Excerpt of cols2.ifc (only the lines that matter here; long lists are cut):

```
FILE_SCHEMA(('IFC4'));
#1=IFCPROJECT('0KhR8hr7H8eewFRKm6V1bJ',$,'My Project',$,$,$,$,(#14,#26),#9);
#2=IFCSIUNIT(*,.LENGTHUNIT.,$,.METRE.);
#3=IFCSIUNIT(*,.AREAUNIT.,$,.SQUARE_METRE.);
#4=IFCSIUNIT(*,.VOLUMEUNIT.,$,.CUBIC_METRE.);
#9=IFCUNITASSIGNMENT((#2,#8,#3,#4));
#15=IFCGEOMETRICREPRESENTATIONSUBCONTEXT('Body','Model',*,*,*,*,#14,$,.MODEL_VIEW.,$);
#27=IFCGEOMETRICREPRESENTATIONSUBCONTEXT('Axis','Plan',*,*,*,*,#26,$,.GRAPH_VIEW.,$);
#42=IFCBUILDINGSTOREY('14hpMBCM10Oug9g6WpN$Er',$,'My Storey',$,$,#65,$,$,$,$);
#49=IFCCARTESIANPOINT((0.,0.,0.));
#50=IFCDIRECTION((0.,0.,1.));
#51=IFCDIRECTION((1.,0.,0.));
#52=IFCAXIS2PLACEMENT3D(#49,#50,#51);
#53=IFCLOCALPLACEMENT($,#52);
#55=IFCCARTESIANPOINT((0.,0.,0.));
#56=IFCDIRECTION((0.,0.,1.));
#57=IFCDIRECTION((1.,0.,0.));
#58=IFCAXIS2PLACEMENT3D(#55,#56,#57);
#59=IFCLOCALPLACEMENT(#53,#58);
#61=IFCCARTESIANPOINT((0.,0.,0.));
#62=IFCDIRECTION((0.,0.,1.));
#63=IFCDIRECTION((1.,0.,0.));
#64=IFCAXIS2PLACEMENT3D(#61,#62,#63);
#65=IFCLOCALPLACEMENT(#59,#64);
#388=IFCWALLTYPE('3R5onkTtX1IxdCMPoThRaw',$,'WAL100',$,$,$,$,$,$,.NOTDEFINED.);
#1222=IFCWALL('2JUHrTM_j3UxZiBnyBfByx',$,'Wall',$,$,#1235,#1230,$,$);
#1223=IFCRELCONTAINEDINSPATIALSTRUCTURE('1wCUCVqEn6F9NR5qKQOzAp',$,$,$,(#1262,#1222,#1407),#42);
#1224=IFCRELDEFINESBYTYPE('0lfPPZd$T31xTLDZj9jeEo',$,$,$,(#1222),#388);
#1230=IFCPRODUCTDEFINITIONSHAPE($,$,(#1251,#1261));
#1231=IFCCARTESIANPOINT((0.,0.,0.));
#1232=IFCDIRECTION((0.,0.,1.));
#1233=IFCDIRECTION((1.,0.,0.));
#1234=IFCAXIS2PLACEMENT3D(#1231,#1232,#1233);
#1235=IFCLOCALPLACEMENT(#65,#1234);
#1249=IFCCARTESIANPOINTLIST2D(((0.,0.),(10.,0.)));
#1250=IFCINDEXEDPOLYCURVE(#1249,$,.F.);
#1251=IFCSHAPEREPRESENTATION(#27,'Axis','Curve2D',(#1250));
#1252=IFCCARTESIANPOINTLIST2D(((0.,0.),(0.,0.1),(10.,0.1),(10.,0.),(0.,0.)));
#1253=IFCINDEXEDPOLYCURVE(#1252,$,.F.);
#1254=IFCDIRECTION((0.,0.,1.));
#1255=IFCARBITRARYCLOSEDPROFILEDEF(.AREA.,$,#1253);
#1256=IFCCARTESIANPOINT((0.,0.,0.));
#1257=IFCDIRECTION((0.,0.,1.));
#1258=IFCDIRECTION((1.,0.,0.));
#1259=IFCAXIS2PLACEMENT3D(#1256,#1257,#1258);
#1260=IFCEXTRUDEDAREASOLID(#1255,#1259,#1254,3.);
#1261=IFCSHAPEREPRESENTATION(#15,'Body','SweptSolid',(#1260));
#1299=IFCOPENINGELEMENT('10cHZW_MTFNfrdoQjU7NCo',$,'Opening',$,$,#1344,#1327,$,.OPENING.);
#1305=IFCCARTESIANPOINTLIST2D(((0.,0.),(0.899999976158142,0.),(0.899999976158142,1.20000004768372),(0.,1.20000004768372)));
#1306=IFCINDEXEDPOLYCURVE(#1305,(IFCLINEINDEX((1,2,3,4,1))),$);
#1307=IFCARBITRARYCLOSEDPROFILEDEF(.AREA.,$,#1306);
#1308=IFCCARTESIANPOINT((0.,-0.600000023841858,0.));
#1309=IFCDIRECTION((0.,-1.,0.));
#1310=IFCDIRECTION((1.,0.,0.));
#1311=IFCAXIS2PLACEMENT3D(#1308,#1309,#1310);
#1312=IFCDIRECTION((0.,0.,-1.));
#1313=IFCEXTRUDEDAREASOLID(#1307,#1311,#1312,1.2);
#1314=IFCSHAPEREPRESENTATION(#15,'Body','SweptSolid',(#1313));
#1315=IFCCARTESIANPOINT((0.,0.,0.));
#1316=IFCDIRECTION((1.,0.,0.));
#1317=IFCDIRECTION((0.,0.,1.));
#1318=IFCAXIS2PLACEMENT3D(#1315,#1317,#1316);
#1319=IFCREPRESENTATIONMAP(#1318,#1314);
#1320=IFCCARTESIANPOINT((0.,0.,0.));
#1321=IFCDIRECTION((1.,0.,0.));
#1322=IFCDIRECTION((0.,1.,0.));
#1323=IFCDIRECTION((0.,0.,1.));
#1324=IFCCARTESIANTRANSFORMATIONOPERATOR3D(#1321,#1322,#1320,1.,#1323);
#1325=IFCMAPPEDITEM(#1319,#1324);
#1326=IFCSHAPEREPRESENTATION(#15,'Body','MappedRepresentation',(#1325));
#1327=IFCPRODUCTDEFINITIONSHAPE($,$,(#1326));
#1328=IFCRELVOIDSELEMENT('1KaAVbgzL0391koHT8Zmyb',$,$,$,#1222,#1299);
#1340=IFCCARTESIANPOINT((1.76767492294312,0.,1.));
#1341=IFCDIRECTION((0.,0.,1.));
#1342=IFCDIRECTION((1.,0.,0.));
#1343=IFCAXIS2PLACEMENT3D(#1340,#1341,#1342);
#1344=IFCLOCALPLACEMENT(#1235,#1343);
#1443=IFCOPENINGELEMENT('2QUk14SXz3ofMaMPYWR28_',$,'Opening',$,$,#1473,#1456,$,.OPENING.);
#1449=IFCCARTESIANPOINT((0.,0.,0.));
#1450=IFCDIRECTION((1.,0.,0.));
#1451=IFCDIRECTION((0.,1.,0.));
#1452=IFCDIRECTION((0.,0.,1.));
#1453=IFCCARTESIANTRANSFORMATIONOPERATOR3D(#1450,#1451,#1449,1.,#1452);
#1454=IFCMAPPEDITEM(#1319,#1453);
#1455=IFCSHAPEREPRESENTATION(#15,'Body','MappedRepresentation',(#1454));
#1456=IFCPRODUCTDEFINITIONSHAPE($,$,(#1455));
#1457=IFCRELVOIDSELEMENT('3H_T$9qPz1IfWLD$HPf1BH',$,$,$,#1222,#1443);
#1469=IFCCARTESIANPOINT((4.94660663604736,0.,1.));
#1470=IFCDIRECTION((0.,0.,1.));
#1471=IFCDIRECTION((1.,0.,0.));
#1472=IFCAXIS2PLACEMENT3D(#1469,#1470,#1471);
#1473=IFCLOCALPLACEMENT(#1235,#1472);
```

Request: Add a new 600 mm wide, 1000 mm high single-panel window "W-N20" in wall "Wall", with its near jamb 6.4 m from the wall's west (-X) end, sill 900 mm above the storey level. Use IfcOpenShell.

```python
import numpy as np
import ifcopenshell
import ifcopenshell.api.feature
import ifcopenshell.api.geometry
import ifcopenshell.api.root
import ifcopenshell.api.spatial
import ifcopenshell.geom
import ifcopenshell.util.element
import ifcopenshell.util.placement
import ifcopenshell.util.representation
import ifcopenshell.util.shape
import ifcopenshell.util.unit

model = ifcopenshell.open("cols2.ifc")
unit_scale = ifcopenshell.util.unit.calculate_unit_scale(model)
settings = ifcopenshell.geom.settings()


def volume(element):
    """Net volume in cubic metres, openings subtracted."""
    shape = ifcopenshell.geom.create_shape(settings, element)
    return ifcopenshell.util.shape.get_volume(shape.geometry)


wall = model.by_guid("2JUHrTM_j3UxZiBnyBfByx")
storey = ifcopenshell.util.element.get_container(wall, ifc_class="IfcBuildingStorey")
context = ifcopenshell.util.representation.get_context(model, "Model", "Body", "MODEL_VIEW")
before = volume(wall)

width, height, from_end, sill = 0.6, 1, 6.4, 0.9  # metres

# The wall runs along its own X axis, and the end named is its -X end.
wall_shape = ifcopenshell.geom.create_shape(settings, wall)
x, y, z = ifcopenshell.util.shape.get_vertices(wall_shape.geometry).T
start = x.min() + from_end
face, thickness = float(y.min()), float(y.max() - y.min())
wall_matrix = ifcopenshell.util.placement.get_local_placement(wall.ObjectPlacement)
level = ifcopenshell.util.placement.get_local_placement(storey.ObjectPlacement)[2, 3]


def in_wall(x, y):
    """Placement at x, y metres in the wall's axes, at sill height."""
    matrix = wall_matrix.copy()
    matrix[:, 3] = wall_matrix @ np.array([x / unit_scale, y / unit_scale, 0.0, 1.0])
    matrix[2, 3] = level + sill / unit_scale
    return matrix


# Opening: a box that overshoots both wall faces by 50 mm.
opening = ifcopenshell.api.root.create_entity(model, ifc_class="IfcOpeningElement", predefined_type="OPENING")
box = ifcopenshell.api.geometry.add_wall_representation(
    model, context=context, length=width, height=height, thickness=thickness + 0.1
)
ifcopenshell.api.geometry.assign_representation(model, product=opening, representation=box)
ifcopenshell.api.geometry.edit_object_placement(model, product=opening, matrix=in_wall(start, face - 0.05), is_si=False)
ifcopenshell.api.feature.add_feature(model, feature=opening, element=wall)

window = ifcopenshell.api.root.create_entity(model, ifc_class="IfcWindow", name="W-N20", predefined_type="WINDOW")
window.OverallWidth, window.OverallHeight = width / unit_scale, height / unit_scale
window.PartitioningType = "SINGLE_PANEL"
body = ifcopenshell.api.geometry.add_window_representation(
    model,
    context=context,
    overall_width=window.OverallWidth,
    overall_height=window.OverallHeight,
    partition_type="SINGLE_PANEL",
)
ifcopenshell.api.geometry.assign_representation(model, product=window, representation=body)
ifcopenshell.api.spatial.assign_container(model, products=[window], relating_structure=storey)
ifcopenshell.api.feature.add_filling(model, opening=opening, element=window)

# Centre the window in the wall's thickness.
ifcopenshell.api.geometry.edit_object_placement(model, product=window, matrix=in_wall(start, face), is_si=False)
window_shape = ifcopenshell.geom.create_shape(settings, window)
depth = ifcopenshell.util.shape.get_vertices(window_shape.geometry)[:, 1]
offset = face + thickness / 2 - (depth.min() + depth.max()) / 2
ifcopenshell.api.geometry.edit_object_placement(model, product=window, matrix=in_wall(start, offset), is_si=False)

after = volume(wall)

print(f"wall volume {before:.3f} -> {after:.3f} m3")

model.write("cols2_rev.ifc")
```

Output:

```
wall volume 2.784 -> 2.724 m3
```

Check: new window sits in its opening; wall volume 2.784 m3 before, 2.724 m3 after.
